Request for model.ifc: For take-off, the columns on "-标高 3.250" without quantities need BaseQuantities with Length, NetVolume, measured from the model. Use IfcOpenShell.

First a look at what the model holds.

```python
import ifcopenshell
import ifcopenshell.util.element
import ifcopenshell.util.unit

model = ifcopenshell.open("model.ifc")
print(model.schema)
for unit_type in ("LENGTHUNIT", "AREAUNIT", "VOLUMEUNIT"):
    print(unit_type, ifcopenshell.util.unit.calculate_unit_scale(model, unit_type))
storey = next(s for s in model.by_type("IfcBuildingStorey") if s.Name == "-标高 3.250")
columns = [e for e in ifcopenshell.util.element.get_decomposition(storey) if e.is_a("IfcColumn")]
for e in sorted(columns, key=lambda e: e.id()):
    print(e.id(), e.is_a(), e.Name, list(ifcopenshell.util.element.get_psets(e, qtos_only=True)), sep=" | ")
```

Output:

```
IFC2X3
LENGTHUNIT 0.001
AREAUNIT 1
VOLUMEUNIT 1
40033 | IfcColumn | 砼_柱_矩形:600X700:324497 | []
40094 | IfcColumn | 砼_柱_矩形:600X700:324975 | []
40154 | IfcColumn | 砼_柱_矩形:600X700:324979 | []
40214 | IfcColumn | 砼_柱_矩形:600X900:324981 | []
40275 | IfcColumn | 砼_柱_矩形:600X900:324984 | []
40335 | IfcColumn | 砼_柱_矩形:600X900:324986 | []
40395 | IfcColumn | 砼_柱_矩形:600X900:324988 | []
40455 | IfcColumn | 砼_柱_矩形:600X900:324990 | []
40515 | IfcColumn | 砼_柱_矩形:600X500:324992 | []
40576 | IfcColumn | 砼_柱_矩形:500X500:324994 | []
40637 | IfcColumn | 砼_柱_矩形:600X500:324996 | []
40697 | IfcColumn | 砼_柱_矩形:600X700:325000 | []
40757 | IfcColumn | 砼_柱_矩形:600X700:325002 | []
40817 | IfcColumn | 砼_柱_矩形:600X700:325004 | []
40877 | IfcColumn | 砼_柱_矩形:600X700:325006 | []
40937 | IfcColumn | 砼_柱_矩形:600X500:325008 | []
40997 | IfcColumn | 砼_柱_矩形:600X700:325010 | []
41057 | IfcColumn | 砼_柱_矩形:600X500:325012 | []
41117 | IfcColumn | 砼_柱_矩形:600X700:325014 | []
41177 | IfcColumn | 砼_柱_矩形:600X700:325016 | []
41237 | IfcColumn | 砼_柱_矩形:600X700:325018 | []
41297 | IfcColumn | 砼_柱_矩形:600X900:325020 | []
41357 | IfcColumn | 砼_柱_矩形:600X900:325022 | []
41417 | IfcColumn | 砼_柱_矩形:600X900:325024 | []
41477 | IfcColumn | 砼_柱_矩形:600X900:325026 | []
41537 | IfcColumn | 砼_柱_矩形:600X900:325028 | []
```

```python
import ifcopenshell
import ifcopenshell.api.pset
import ifcopenshell.geom
import ifcopenshell.util.element
import ifcopenshell.util.shape
import ifcopenshell.util.unit

model = ifcopenshell.open("model.ifc")
unit_scale = ifcopenshell.util.unit.calculate_unit_scale(model)
volume_scale = ifcopenshell.util.unit.calculate_unit_scale(model, "VOLUMEUNIT")
settings = ifcopenshell.geom.settings()

storey = next(s for s in model.by_type("IfcBuildingStorey") if s.Name == "-标高 3.250")
columns = [e for e in ifcopenshell.util.element.get_decomposition(storey) if e.is_a("IfcColumn")]

for e in sorted(columns, key=lambda e: e.id()):
    if ifcopenshell.util.element.get_psets(e, qtos_only=True, should_inherit=False):
        continue
    # Geometry comes back in metres, in the element's own axes.
    shape = ifcopenshell.geom.create_shape(settings, e)
    values = {
        "Length": ifcopenshell.util.shape.get_z(shape.geometry) / unit_scale,
        "NetVolume": ifcopenshell.util.shape.get_volume(shape.geometry) / volume_scale,
    }
    qto = ifcopenshell.api.pset.add_qto(model, product=e, name="BaseQuantities")
    ifcopenshell.api.pset.edit_qto(model, qto=qto, properties=values)
    print(e.id(), {k: round(v, 3) for k, v in values.items()})

model.write("model-out.ifc")
```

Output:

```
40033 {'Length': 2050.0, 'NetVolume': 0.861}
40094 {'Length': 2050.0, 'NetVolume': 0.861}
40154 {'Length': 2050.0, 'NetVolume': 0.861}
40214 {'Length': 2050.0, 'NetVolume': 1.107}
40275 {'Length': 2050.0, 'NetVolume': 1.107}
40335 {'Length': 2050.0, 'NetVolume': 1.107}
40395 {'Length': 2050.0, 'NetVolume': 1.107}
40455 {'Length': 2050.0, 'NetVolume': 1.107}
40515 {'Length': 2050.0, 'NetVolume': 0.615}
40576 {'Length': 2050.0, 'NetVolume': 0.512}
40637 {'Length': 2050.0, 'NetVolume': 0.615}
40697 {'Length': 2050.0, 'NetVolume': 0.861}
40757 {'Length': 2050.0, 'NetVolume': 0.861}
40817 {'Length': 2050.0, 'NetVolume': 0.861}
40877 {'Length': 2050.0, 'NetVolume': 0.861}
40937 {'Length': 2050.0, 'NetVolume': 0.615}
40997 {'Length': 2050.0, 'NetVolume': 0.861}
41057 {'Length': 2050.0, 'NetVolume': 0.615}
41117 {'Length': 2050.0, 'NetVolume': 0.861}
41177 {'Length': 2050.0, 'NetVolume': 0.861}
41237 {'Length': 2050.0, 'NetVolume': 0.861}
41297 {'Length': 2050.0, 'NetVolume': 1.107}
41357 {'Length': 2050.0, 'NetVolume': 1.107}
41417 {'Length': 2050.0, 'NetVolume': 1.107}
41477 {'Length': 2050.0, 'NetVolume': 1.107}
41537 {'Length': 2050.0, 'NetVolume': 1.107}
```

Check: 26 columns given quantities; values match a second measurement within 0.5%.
